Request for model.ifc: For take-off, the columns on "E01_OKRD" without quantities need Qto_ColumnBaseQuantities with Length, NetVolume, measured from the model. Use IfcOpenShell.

First a look at what the model holds.

```python
import ifcopenshell
import ifcopenshell.util.element
import ifcopenshell.util.unit

model = ifcopenshell.open("model.ifc")
print(model.schema)
for unit_type in ("LENGTHUNIT", "AREAUNIT", "VOLUMEUNIT"):
    print(unit_type, ifcopenshell.util.unit.calculate_unit_scale(model, unit_type))
storey = next(s for s in model.by_type("IfcBuildingStorey") if s.Name == "E01_OKRD")
columns = [e for e in ifcopenshell.util.element.get_decomposition(storey) if e.is_a("IfcColumn")]
for e in sorted(columns, key=lambda e: e.id()):
    print(e.id(), e.is_a(), e.Name, list(ifcopenshell.util.element.get_psets(e, qtos_only=True)), sep=" | ")
```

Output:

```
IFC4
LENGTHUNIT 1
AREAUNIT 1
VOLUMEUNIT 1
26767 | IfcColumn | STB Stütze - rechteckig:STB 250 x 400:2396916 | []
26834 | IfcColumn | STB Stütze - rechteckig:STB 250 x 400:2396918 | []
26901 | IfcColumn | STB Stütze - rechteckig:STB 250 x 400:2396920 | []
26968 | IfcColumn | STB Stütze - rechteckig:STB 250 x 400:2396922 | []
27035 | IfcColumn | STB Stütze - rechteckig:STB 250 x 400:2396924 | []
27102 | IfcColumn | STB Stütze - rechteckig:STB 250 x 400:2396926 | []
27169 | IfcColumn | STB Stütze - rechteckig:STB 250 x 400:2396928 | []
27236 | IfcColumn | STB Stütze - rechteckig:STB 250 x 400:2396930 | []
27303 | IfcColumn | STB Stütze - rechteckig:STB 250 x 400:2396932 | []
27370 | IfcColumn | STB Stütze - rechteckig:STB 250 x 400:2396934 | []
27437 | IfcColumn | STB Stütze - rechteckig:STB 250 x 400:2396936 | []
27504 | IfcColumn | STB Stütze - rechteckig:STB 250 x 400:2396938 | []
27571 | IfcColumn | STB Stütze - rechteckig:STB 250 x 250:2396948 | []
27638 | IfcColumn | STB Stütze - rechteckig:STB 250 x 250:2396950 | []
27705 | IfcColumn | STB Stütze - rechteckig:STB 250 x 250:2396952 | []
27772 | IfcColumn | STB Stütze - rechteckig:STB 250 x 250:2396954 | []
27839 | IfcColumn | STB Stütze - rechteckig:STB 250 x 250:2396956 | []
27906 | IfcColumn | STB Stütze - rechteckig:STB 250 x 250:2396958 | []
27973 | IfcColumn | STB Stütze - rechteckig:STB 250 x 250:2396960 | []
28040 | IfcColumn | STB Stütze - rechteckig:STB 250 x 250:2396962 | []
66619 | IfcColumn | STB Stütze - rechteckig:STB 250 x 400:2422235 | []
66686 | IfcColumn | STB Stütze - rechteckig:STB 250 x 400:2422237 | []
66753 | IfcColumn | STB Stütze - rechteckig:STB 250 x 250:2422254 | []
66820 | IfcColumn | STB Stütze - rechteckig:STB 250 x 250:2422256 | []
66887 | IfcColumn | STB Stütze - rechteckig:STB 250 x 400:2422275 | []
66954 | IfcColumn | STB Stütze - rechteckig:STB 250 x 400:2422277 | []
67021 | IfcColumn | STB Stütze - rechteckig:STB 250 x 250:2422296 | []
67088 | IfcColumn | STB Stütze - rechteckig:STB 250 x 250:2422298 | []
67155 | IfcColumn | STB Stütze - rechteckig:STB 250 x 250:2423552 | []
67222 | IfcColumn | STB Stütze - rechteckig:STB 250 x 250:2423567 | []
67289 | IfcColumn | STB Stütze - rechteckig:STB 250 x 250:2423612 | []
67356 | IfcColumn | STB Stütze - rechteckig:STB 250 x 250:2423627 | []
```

```python
import ifcopenshell
import ifcopenshell.api.pset
import ifcopenshell.geom
import ifcopenshell.util.element
import ifcopenshell.util.shape
import ifcopenshell.util.unit

model = ifcopenshell.open("model.ifc")
unit_scale = ifcopenshell.util.unit.calculate_unit_scale(model)
volume_scale = ifcopenshell.util.unit.calculate_unit_scale(model, "VOLUMEUNIT")
settings = ifcopenshell.geom.settings()

storey = next(s for s in model.by_type("IfcBuildingStorey") if s.Name == "E01_OKRD")
columns = [e for e in ifcopenshell.util.element.get_decomposition(storey) if e.is_a("IfcColumn")]

for e in sorted(columns, key=lambda e: e.id()):
    if ifcopenshell.util.element.get_psets(e, qtos_only=True, should_inherit=False):
        continue
    # Geometry comes back in metres, in the element's own axes.
    shape = ifcopenshell.geom.create_shape(settings, e)
    values = {
        "Length": ifcopenshell.util.shape.get_z(shape.geometry) / unit_scale,
        "NetVolume": ifcopenshell.util.shape.get_volume(shape.geometry) / volume_scale,
    }
    qto = ifcopenshell.api.pset.add_qto(model, product=e, name="Qto_ColumnBaseQuantities")
    ifcopenshell.api.pset.edit_qto(model, qto=qto, properties=values)
    print(e.id(), {k: round(v, 3) for k, v in values.items()})

model.write("model-out.ifc")
```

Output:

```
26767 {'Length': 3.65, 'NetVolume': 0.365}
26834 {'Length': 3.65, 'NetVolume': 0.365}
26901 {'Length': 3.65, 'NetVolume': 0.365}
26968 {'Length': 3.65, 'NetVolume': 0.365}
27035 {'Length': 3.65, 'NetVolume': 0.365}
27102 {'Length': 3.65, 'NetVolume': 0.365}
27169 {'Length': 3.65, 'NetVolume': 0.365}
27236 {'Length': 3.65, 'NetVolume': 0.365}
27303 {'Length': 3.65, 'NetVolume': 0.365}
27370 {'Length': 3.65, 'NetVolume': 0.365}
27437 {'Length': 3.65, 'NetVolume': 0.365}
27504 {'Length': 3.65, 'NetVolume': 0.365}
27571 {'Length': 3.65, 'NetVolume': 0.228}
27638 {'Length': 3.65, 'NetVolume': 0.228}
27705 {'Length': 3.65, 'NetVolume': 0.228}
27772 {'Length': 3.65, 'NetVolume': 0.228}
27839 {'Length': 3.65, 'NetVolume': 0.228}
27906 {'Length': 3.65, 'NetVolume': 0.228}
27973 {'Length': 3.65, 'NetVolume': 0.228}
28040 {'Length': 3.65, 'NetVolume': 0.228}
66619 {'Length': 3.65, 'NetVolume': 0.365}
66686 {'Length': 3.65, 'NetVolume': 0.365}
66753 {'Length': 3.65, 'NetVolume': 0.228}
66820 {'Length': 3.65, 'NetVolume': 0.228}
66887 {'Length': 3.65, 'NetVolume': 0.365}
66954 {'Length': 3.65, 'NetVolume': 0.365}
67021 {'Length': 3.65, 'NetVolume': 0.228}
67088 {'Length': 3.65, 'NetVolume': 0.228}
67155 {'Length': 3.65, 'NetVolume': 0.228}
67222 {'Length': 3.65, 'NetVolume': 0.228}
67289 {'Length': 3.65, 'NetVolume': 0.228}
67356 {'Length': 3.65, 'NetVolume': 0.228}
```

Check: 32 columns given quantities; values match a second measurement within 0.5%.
